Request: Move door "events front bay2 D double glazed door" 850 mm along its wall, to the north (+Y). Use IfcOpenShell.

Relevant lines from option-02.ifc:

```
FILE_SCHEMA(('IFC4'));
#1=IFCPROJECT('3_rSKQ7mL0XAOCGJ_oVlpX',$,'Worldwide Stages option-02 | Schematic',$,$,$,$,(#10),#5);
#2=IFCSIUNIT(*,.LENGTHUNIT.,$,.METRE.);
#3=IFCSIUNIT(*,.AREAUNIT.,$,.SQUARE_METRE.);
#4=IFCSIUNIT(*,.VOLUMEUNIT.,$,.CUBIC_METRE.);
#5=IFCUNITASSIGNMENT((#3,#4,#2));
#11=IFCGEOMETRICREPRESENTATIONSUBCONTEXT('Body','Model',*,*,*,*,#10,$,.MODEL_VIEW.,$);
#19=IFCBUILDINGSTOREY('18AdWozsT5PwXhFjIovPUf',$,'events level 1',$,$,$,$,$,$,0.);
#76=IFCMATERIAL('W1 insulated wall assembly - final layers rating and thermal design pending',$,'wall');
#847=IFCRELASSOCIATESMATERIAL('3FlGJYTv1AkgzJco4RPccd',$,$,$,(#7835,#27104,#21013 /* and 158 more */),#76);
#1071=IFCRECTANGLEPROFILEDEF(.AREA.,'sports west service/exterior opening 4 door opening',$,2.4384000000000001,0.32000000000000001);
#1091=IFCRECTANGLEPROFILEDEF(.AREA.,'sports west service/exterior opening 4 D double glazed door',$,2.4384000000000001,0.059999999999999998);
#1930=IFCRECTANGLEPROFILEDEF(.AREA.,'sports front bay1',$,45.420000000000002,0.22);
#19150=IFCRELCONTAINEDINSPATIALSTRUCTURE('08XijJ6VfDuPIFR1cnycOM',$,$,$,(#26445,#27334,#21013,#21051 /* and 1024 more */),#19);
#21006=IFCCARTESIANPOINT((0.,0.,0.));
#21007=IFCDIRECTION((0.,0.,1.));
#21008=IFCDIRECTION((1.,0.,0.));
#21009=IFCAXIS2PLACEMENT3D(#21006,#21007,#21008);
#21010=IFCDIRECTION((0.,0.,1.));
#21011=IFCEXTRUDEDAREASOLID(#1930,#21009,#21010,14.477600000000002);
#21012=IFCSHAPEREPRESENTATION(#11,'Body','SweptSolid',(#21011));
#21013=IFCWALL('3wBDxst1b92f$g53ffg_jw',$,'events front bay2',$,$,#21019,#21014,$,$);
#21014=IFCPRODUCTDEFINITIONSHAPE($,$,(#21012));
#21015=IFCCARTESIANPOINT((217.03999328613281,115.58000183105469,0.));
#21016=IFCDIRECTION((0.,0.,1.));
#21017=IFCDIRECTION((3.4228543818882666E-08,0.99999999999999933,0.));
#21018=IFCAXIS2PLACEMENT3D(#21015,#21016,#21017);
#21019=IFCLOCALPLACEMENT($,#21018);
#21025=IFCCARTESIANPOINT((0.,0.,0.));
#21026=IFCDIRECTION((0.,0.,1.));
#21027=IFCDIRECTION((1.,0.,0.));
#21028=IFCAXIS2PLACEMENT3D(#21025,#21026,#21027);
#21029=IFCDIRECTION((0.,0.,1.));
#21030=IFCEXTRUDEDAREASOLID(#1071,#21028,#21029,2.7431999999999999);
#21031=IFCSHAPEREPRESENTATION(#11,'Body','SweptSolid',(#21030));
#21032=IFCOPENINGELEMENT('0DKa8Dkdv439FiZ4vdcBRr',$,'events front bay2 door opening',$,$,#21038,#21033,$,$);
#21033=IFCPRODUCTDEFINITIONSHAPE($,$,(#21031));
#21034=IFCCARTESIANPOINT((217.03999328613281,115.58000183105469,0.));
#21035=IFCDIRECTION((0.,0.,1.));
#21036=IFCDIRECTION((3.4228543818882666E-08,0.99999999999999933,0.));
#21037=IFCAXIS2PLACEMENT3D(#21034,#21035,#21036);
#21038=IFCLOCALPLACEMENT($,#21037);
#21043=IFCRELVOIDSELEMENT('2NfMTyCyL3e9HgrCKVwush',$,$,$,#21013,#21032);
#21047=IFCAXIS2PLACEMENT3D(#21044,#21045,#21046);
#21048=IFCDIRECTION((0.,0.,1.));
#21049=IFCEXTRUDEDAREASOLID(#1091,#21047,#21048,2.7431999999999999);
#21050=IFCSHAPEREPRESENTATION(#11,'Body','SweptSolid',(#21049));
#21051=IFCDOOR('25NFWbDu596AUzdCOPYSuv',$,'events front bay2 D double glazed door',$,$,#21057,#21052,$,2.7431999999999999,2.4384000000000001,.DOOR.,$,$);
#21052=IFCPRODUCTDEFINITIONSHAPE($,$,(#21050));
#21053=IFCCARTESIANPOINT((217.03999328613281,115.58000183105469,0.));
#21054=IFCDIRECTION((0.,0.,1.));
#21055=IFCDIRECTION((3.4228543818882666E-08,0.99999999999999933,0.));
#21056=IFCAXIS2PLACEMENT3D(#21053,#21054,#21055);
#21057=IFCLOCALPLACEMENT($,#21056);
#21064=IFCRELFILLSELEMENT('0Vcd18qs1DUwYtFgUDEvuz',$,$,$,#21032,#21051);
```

```python
import ifcopenshell
import ifcopenshell.api.geometry
import ifcopenshell.util.placement
import ifcopenshell.util.unit

model = ifcopenshell.open("option-02.ifc")
unit_scale = ifcopenshell.util.unit.calculate_unit_scale(model)

door = model.by_id(21051)
opening = door.FillsVoids[0].RelatingOpeningElement
wall = opening.VoidsElements[0].RelatingBuildingElement

wall_matrix = ifcopenshell.util.placement.get_local_placement(wall.ObjectPlacement)
shift = wall_matrix[:3, 0] * 0.85 / unit_scale
before = ifcopenshell.util.placement.get_local_placement(door.ObjectPlacement)[:3, 3].copy()

# The door is not placed relative to its opening, so move both.
for product in (opening, door):
    matrix = ifcopenshell.util.placement.get_local_placement(product.ObjectPlacement)
    matrix[:3, 3] += shift
    ifcopenshell.api.geometry.edit_object_placement(model, product=product, matrix=matrix, is_si=False)

after = ifcopenshell.util.placement.get_local_placement(door.ObjectPlacement)[:3, 3]
print("door moved by", (after - before).round(3) + 0.0)

model.write("option-02_edited.ifc")
```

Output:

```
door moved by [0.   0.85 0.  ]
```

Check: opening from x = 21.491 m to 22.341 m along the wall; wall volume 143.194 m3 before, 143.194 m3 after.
